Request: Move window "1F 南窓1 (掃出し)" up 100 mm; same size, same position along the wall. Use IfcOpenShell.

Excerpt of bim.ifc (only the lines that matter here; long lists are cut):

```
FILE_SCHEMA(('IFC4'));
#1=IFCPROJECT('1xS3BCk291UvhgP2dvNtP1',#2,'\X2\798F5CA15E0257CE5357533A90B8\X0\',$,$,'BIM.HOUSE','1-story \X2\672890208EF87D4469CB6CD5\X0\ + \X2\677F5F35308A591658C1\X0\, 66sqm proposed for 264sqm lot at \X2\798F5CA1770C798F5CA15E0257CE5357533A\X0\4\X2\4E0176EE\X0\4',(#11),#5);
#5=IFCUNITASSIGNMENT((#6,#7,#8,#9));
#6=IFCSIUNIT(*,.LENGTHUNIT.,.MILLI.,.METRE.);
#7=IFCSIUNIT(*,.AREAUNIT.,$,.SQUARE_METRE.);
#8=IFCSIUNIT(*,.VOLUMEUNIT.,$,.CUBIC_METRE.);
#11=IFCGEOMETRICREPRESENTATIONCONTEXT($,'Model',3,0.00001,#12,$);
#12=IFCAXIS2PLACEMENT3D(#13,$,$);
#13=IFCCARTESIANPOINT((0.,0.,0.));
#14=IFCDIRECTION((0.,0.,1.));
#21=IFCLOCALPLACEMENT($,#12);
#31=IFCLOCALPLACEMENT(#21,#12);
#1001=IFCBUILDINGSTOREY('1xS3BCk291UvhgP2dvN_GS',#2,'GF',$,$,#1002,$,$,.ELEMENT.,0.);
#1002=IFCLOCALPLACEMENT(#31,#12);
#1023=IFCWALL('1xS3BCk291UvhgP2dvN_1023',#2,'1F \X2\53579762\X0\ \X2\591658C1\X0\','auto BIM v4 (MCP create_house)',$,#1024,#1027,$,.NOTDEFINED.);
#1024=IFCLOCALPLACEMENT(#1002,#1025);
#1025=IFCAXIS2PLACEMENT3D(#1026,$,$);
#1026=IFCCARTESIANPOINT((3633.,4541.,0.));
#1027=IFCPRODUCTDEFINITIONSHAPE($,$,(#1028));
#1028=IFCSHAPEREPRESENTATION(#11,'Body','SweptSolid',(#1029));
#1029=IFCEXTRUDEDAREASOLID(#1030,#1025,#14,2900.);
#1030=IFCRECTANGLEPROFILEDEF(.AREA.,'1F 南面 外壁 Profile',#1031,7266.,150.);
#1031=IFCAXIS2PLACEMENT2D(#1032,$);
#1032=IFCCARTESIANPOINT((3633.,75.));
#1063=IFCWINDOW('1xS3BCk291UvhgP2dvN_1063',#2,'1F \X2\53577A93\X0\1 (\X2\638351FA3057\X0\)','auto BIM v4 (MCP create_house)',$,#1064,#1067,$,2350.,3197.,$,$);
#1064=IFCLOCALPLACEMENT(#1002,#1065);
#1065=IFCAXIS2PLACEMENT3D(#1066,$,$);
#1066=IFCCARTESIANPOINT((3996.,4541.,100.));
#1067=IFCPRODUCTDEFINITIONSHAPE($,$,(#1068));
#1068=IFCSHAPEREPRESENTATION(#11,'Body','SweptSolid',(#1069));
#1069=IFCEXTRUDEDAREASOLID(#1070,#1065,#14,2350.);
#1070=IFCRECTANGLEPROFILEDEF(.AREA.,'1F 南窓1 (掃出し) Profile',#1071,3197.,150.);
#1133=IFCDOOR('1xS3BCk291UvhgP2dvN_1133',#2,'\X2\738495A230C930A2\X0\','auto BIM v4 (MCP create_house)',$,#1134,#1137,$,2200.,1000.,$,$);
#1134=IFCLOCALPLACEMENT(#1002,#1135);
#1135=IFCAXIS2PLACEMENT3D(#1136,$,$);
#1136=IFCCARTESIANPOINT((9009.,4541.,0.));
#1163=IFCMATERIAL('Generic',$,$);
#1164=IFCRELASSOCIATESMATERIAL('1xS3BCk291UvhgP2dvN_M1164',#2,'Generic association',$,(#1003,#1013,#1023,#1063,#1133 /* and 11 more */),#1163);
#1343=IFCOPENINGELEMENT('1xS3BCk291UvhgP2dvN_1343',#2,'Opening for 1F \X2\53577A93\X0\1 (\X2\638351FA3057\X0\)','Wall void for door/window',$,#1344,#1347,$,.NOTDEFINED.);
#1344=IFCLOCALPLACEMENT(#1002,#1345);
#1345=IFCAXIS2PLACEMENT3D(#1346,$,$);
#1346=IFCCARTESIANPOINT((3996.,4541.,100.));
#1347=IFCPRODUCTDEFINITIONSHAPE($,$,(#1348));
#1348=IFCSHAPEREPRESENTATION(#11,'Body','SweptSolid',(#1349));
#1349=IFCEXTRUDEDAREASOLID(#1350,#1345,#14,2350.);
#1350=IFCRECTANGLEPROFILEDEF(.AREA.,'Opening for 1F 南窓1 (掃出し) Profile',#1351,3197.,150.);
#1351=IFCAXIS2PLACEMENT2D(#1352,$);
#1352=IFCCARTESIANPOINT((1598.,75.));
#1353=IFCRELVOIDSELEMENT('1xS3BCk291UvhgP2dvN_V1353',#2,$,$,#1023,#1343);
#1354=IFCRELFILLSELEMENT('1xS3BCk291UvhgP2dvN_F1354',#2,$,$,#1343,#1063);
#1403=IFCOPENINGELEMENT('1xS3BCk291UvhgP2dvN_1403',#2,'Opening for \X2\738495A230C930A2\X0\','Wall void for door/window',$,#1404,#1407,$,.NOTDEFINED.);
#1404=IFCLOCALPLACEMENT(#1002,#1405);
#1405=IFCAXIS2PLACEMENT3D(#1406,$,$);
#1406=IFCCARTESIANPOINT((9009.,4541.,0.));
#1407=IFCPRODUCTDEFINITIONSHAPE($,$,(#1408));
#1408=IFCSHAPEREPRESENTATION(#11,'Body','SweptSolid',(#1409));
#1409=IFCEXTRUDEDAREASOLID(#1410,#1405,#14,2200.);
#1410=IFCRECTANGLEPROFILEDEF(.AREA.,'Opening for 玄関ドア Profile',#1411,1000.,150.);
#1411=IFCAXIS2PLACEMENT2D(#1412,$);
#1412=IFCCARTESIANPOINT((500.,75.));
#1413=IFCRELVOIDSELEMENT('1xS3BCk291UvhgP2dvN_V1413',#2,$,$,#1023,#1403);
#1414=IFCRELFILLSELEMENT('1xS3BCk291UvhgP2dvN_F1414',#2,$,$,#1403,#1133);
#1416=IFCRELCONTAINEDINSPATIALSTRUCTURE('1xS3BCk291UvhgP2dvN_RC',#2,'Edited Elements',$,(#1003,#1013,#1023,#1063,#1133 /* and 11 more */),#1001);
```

```python
import numpy as np
import ifcopenshell
import ifcopenshell.api.geometry
import ifcopenshell.util.placement
import ifcopenshell.util.unit

model = ifcopenshell.open("bim.ifc")
unit_scale = ifcopenshell.util.unit.calculate_unit_scale(model)

window = model.by_guid("1xS3BCk291UvhgP2dvN_1063")
opening = window.FillsVoids[0].RelatingOpeningElement
dz = 0.1 / unit_scale

shift = np.array([0.0, 0.0, dz])
# The window is not placed relative to its opening, so move both.
for product in (opening, window):
    matrix = ifcopenshell.util.placement.get_local_placement(product.ObjectPlacement)
    matrix[:3, 3] += shift
    ifcopenshell.api.geometry.edit_object_placement(model, product=product, matrix=matrix, is_si=False)

print(f"moved by {dz * unit_scale:+.3f} m")

model.write("bim_updated.ifc")
```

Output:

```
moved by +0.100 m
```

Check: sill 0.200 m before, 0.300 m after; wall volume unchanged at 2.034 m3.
